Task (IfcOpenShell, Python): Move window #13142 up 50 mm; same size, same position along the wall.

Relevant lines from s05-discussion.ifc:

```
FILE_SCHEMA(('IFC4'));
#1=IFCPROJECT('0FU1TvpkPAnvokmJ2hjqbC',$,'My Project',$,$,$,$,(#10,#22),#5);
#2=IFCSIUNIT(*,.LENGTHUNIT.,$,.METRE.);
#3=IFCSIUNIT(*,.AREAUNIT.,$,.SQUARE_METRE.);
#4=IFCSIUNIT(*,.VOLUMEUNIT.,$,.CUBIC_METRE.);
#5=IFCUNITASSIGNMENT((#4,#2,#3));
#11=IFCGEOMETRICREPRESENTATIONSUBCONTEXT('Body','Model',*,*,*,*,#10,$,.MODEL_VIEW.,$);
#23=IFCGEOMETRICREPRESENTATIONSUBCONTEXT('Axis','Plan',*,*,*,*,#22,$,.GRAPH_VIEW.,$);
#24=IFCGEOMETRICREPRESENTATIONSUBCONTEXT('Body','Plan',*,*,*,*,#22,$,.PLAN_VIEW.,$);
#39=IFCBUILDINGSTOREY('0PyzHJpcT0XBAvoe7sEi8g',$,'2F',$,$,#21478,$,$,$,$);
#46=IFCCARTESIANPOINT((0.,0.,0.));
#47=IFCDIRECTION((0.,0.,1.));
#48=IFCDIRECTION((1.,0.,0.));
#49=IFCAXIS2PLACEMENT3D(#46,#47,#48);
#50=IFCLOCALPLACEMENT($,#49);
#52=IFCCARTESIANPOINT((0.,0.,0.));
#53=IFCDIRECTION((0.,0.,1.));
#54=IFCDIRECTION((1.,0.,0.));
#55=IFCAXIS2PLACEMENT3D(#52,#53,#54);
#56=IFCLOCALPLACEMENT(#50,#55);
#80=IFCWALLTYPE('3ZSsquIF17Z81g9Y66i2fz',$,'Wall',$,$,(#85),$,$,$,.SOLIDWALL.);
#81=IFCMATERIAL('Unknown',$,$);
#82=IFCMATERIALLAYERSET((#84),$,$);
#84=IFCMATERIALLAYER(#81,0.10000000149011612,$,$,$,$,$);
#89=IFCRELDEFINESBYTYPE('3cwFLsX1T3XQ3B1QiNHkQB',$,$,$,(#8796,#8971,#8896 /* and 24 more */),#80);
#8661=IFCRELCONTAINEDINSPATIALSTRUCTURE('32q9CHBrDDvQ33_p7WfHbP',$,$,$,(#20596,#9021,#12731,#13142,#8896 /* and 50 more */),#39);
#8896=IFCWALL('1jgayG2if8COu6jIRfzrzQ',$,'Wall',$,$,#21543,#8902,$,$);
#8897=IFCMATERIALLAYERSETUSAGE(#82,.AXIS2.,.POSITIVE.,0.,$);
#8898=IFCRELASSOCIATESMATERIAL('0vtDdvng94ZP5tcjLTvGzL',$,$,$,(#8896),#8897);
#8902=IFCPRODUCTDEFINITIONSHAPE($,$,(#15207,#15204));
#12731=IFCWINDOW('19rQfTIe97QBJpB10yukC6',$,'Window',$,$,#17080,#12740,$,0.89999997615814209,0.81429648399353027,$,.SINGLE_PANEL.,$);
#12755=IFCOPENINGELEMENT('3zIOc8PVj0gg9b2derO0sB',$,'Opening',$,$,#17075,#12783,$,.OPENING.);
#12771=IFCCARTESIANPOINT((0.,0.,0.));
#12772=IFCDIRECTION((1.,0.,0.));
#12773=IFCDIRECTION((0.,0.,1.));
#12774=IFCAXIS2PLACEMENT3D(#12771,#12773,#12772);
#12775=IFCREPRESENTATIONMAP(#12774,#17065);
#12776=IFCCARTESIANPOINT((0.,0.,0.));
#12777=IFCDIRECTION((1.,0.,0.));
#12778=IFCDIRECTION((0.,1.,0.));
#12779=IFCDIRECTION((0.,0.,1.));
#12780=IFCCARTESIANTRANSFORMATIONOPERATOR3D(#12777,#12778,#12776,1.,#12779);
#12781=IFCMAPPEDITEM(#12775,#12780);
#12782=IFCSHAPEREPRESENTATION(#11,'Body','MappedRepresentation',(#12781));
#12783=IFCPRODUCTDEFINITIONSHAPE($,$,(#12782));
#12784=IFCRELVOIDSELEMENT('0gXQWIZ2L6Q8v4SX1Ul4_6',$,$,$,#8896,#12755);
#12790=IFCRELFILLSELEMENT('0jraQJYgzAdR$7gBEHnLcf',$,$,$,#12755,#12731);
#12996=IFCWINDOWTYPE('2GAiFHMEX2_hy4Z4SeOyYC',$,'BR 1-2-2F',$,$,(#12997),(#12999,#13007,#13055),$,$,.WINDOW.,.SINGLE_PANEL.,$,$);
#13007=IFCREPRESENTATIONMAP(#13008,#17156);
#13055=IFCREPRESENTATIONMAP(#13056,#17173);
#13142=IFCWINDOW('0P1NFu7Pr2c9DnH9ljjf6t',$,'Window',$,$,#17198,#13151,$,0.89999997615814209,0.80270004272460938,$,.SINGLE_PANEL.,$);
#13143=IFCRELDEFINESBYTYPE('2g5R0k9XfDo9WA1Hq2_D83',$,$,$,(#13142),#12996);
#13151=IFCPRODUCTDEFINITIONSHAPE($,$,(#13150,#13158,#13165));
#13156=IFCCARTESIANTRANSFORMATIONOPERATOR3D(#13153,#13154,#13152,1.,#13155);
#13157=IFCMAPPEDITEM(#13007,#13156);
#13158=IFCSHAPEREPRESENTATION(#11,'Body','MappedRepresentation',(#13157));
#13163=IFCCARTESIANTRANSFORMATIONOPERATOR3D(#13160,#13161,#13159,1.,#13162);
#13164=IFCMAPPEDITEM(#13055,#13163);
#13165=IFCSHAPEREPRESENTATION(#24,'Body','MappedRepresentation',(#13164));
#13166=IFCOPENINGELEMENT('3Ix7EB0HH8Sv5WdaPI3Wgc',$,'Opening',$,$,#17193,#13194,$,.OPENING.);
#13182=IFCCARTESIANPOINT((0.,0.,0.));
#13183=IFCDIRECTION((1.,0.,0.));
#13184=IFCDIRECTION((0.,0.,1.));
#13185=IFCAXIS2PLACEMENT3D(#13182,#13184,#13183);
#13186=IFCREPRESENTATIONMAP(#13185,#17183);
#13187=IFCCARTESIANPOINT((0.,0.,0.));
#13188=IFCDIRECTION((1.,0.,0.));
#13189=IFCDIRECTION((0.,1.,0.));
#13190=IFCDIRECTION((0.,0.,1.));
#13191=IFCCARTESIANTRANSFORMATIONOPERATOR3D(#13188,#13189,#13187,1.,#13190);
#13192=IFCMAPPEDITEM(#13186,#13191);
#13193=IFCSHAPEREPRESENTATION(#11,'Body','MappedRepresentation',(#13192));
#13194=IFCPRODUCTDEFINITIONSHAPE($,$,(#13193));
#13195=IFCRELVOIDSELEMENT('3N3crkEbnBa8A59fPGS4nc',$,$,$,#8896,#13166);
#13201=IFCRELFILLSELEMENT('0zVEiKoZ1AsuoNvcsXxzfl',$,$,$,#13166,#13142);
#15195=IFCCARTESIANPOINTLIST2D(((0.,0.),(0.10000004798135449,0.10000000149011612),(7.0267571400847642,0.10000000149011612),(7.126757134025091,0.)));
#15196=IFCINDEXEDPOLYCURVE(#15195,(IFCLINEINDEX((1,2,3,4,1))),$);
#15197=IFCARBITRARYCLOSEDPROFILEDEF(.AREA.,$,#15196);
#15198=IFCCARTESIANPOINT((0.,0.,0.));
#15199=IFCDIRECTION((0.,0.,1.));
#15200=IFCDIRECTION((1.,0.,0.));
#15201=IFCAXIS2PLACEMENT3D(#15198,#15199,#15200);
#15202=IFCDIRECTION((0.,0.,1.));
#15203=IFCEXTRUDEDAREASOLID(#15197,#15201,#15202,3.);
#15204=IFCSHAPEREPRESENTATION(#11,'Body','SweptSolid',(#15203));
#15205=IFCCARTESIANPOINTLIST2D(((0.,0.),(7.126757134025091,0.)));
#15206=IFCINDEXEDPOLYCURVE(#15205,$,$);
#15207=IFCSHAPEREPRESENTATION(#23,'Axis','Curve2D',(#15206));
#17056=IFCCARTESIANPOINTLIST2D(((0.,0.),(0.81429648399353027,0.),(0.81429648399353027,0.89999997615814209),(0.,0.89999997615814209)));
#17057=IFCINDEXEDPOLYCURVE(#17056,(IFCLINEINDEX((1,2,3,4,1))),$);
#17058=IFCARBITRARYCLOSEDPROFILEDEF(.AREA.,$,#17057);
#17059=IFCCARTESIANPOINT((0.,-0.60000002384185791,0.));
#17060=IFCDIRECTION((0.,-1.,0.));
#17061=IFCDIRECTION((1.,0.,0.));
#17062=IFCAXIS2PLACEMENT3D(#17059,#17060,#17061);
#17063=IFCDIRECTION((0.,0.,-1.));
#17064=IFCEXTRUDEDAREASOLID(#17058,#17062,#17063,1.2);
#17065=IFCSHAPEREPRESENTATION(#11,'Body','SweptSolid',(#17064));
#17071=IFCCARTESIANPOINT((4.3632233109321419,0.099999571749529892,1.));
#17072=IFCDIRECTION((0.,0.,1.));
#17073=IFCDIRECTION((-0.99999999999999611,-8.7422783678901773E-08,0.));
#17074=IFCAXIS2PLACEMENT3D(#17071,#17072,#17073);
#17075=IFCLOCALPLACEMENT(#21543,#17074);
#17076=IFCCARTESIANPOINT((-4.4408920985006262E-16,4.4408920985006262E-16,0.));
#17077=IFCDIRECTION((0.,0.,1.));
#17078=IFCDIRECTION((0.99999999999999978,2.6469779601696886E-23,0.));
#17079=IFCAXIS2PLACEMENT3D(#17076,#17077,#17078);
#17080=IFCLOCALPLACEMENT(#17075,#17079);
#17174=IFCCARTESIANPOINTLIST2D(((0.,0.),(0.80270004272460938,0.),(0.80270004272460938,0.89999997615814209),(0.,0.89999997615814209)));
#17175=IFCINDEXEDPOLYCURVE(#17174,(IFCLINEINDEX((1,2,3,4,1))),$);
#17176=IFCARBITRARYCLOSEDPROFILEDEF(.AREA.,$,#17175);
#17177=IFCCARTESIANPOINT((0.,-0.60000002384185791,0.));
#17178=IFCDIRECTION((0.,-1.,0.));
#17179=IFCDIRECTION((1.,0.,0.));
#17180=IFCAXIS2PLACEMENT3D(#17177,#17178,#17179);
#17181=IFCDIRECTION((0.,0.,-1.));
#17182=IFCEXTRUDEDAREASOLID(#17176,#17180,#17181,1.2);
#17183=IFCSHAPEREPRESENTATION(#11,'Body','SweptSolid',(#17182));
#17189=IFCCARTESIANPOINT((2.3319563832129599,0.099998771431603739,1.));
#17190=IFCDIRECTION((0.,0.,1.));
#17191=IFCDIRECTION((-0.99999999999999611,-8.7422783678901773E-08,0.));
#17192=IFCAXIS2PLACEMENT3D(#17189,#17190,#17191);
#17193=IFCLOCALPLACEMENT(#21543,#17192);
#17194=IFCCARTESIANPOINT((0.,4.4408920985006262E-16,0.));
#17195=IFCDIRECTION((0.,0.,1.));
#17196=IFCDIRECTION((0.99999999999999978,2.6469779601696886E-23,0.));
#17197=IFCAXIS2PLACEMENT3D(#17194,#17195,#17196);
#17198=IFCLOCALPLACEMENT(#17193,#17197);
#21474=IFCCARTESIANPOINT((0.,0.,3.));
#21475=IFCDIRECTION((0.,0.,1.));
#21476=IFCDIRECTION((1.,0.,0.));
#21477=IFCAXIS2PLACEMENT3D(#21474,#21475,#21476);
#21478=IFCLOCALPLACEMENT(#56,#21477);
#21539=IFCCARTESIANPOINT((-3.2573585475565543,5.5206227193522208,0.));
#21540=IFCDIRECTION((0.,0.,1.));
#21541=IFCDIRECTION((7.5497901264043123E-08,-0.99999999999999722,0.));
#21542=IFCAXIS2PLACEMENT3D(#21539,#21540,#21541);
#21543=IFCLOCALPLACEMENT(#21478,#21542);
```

```python
import numpy as np
import ifcopenshell
import ifcopenshell.api.geometry
import ifcopenshell.util.placement
import ifcopenshell.util.unit

model = ifcopenshell.open("s05-discussion.ifc")
unit_scale = ifcopenshell.util.unit.calculate_unit_scale(model)

window = model.by_id(13142)
opening = window.FillsVoids[0].RelatingOpeningElement
dz = 0.05

shift = np.array([0.0, 0.0, dz])
# The window is placed relative to its opening, so it follows when the opening moves.
matrix = ifcopenshell.util.placement.get_local_placement(opening.ObjectPlacement)
matrix[:3, 3] += shift
ifcopenshell.api.geometry.edit_object_placement(
    model, product=opening, matrix=matrix, is_si=False, should_transform_children=True
)

print(f"moved by {dz * unit_scale:+.3f} m")

model.write("s05-discussion-out.ifc")
```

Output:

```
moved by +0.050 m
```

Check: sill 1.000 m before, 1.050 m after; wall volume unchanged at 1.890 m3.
